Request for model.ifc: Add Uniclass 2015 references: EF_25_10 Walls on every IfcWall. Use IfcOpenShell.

First a look at what the model holds.

```python
import ifcopenshell

model = ifcopenshell.open("model.ifc")
print(model.schema)
print("classifications:", [c.Name for c in model.by_type("IfcClassification")])
for ifc_class in ("IfcDoor", "IfcRoof", "IfcStair", "IfcWall", "IfcWindow"):
    print(ifc_class, len(model.by_type(ifc_class)))
```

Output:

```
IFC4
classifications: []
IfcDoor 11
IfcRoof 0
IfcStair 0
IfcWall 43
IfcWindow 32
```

```python
import ifcopenshell
import ifcopenshell.api.classification

model = ifcopenshell.open("model.ifc")

system = ifcopenshell.api.classification.add_classification(model, classification="Uniclass 2015")

codes = {
    "IfcWall": ("EF_25_10", "Walls"),
}
for ifc_class, (code, name) in codes.items():
    products = model.by_type(ifc_class)
    ifcopenshell.api.classification.add_reference(
        model, products=products, classification=system, identification=code, name=name
    )
    print(code, len(products))

model.write("model_rev.ifc")
```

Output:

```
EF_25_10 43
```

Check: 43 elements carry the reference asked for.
